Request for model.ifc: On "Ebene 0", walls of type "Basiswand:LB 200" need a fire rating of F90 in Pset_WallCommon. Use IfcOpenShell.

First a look at what the model holds.

```python
import ifcopenshell
import ifcopenshell.util.element

model = ifcopenshell.open("model.ifc")
print(model.schema)
storey = next(s for s in model.by_type("IfcBuildingStorey") if s.Name == "Ebene 0")
walls = [e for e in ifcopenshell.util.element.get_decomposition(storey) if e.is_a("IfcWall")]
seen = {}
for e in walls:
    element_type = ifcopenshell.util.element.get_type(e)
    key = (element_type.Name if element_type != e and element_type else None, ifcopenshell.util.element.get_pset(e, "Pset_WallCommon", "FireRating"))
    seen[key] = seen.get(key, 0) + 1
for (name, value), count in sorted(seen.items(), key=str):
    print(count, "x", name, "|", value)
```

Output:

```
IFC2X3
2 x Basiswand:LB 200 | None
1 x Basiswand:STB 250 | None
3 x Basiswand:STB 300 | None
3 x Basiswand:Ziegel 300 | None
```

```python
import ifcopenshell
import ifcopenshell.api.pset
import ifcopenshell.util.element

model = ifcopenshell.open("model.ifc")

storey = next(s for s in model.by_type("IfcBuildingStorey") if s.Name == "Ebene 0")
walls = [e for e in ifcopenshell.util.element.get_decomposition(storey) if e.is_a("IfcWall")]

count = 0
for e in walls:
    element_type = ifcopenshell.util.element.get_type(e)
    if element_type in (None, e) or element_type.Name != "Basiswand:LB 200":
        continue
    # add_pset returns the element's existing set when there is one.
    pset = ifcopenshell.api.pset.add_pset(model, product=e, name="Pset_WallCommon")
    ifcopenshell.api.pset.edit_pset(model, pset=pset, properties={"FireRating": "F90"})
    count += 1

print(count, "walls updated")

model.write("model_updated.ifc")
```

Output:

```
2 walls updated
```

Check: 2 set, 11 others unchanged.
